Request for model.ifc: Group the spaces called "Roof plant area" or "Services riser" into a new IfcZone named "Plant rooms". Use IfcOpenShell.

First a look at what the model holds.

```python
import ifcopenshell

model = ifcopenshell.open("model.ifc")
print(model.schema)
seen = {}
for space in model.by_type("IfcSpace"):
    seen[space.LongName] = seen.get(space.LongName, 0) + 1
for name, count in sorted(seen.items(), key=str):
    print(count, "x", name)
print("zones:", [z.Name for z in model.by_type("IfcZone")][:20])
```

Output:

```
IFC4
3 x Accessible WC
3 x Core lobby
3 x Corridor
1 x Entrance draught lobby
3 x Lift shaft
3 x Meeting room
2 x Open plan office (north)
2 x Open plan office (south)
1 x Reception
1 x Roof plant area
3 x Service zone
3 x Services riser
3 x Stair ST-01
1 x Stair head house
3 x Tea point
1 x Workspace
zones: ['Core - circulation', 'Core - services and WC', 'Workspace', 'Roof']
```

```python
import ifcopenshell
import ifcopenshell.api.group
import ifcopenshell.api.root

model = ifcopenshell.open("model.ifc")

names = {"Roof plant area", "Services riser"}
spaces = [s for s in model.by_type("IfcSpace") if s.LongName in names]

zone = ifcopenshell.api.root.create_entity(model, ifc_class="IfcZone", name="Plant rooms")
ifcopenshell.api.group.assign_group(model, products=spaces, group=zone)
print(len(spaces), "spaces in", zone.Name)

model.write("model-out.ifc")
```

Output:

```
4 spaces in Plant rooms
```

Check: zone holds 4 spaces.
